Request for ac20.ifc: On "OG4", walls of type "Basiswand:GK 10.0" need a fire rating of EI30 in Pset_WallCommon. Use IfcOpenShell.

First a look at what the model holds.

```python
import ifcopenshell
import ifcopenshell.util.element

model = ifcopenshell.open("ac20.ifc")
print(model.schema)
storey = next(s for s in model.by_type("IfcBuildingStorey") if s.Name == "OG4")
walls = [e for e in ifcopenshell.util.element.get_decomposition(storey) if e.is_a("IfcWall")]
seen = {}
for e in walls:
    element_type = ifcopenshell.util.element.get_type(e)
    key = (element_type.Name if element_type != e and element_type else None, ifcopenshell.util.element.get_pset(e, "Pset_WallCommon", "FireRating"))
    seen[key] = seen.get(key, 0) + 1
for (name, value), count in sorted(seen.items(), key=str):
    print(count, "x", name, "|", value)
```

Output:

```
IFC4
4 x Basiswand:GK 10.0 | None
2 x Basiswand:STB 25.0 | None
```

```python
import ifcopenshell
import ifcopenshell.api.pset
import ifcopenshell.util.element

model = ifcopenshell.open("ac20.ifc")

storey = next(s for s in model.by_type("IfcBuildingStorey") if s.Name == "OG4")
walls = [e for e in ifcopenshell.util.element.get_decomposition(storey) if e.is_a("IfcWall")]

count = 0
for e in walls:
    element_type = ifcopenshell.util.element.get_type(e)
    if element_type in (None, e) or element_type.Name != "Basiswand:GK 10.0":
        continue
    # add_pset returns the element's existing set when there is one.
    pset = ifcopenshell.api.pset.add_pset(model, product=e, name="Pset_WallCommon")
    ifcopenshell.api.pset.edit_pset(model, pset=pset, properties={"FireRating": "EI30"})
    count += 1

print(count, "walls updated")

model.write("ac20_rev.ifc")
```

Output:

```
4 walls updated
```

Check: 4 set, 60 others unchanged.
